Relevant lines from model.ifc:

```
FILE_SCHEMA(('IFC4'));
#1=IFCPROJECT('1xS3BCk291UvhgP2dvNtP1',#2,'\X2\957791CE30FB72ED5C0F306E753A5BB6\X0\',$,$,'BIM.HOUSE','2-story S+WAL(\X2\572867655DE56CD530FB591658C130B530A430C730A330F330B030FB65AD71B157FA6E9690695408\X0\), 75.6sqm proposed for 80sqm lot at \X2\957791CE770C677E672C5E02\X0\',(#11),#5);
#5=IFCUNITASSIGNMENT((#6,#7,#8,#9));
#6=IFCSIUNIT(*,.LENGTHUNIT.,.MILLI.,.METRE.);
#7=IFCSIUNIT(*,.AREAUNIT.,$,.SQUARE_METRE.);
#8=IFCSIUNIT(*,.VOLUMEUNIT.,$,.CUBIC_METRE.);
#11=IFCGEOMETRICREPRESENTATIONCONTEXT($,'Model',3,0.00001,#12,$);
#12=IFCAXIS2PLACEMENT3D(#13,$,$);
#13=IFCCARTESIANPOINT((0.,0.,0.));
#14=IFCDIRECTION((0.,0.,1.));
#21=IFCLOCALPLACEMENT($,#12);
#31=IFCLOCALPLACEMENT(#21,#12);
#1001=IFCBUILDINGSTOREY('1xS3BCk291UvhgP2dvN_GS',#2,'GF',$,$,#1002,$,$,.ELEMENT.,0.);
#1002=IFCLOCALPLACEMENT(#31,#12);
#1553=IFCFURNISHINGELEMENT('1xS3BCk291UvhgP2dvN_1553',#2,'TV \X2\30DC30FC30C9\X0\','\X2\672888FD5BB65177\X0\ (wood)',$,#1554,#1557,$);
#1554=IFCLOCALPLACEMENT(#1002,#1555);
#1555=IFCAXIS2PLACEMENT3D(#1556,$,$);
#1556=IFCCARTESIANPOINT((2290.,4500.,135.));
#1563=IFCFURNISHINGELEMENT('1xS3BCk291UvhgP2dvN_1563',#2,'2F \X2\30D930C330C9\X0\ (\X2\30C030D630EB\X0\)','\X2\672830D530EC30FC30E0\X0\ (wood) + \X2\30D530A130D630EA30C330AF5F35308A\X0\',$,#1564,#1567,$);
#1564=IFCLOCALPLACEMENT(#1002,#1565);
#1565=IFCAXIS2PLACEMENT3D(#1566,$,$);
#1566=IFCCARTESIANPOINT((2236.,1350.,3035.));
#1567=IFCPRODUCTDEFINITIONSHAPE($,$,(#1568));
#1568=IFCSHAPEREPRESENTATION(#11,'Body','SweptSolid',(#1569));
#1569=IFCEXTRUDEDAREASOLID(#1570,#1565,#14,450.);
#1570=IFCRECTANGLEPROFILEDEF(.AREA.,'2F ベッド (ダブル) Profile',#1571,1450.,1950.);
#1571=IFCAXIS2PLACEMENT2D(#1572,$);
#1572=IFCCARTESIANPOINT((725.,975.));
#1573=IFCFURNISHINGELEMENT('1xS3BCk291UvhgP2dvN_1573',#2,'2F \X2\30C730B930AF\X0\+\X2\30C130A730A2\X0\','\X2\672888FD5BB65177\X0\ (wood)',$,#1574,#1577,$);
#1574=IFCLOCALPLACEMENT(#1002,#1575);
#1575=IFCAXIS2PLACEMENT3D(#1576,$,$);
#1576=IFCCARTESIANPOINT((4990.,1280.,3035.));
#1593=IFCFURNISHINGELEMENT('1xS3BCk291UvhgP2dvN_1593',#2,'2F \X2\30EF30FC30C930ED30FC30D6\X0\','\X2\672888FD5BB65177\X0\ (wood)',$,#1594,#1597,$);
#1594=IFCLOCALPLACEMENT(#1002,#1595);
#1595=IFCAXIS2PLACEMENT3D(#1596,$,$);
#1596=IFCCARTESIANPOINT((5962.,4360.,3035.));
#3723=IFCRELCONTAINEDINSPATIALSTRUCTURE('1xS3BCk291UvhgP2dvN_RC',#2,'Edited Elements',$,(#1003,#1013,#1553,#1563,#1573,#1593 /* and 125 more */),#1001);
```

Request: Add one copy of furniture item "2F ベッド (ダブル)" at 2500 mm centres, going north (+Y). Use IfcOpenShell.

```python
import numpy as np
import ifcopenshell
import ifcopenshell.api.geometry
import ifcopenshell.api.root
import ifcopenshell.util.element
import ifcopenshell.util.placement

model = ifcopenshell.open("model.ifc")


def reuse_history(source, copy):
    """copy_class also copies each property set's owner history, people and application; keep the originals."""
    for rel in copy.IsDefinedBy:
        if rel.is_a("IfcRelDefinesByProperties") and (history := rel.RelatingPropertyDefinition.OwnerHistory):
            rel.RelatingPropertyDefinition.OwnerHistory = source.OwnerHistory
            ifcopenshell.util.element.remove_deep2(model, history)


source = model.by_guid("1xS3BCk291UvhgP2dvN_1563")
base = ifcopenshell.util.placement.get_local_placement(source.ObjectPlacement)
step = np.array([0.0, 1.0, 0.0]) * 2500.0

for i in range(1, 2):
    copy = ifcopenshell.api.root.copy_class(model, product=source)
    copy.Representation = ifcopenshell.util.element.copy_deep(
        model, source.Representation, exclude=["IfcGeometricRepresentationContext", "IfcRepresentationMap"]
    )
    reuse_history(source, copy)
    matrix = base.copy()
    matrix[:3, 3] += i * step
    print("added at", matrix[:3, 3].round(3) + 0.0)
    ifcopenshell.api.geometry.edit_object_placement(model, product=copy, matrix=matrix, is_si=False)

model.write("model_edited.ifc")
```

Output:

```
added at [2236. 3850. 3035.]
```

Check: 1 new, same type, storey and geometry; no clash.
